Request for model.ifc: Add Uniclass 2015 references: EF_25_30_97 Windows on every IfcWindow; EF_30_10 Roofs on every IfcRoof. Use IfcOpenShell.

First a look at what the model holds.

```python
import ifcopenshell

model = ifcopenshell.open("model.ifc")
print(model.schema)
print("classifications:", [c.Name for c in model.by_type("IfcClassification")])
for ifc_class in ("IfcDoor", "IfcRoof", "IfcStair", "IfcWall", "IfcWindow"):
    print(ifc_class, len(model.by_type(ifc_class)))
```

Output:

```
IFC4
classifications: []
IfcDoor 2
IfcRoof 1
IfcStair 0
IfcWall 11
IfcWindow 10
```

```python
import ifcopenshell
import ifcopenshell.api.classification

model = ifcopenshell.open("model.ifc")

system = ifcopenshell.api.classification.add_classification(model, classification="Uniclass 2015")

codes = {
    "IfcWindow": ("EF_25_30_97", "Windows"),
    "IfcRoof": ("EF_30_10", "Roofs"),
}
for ifc_class, (code, name) in codes.items():
    products = model.by_type(ifc_class)
    ifcopenshell.api.classification.add_reference(
        model, products=products, classification=system, identification=code, name=name
    )
    print(code, len(products))

model.write("model_updated.ifc")
```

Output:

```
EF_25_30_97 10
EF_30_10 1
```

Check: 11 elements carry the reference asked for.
